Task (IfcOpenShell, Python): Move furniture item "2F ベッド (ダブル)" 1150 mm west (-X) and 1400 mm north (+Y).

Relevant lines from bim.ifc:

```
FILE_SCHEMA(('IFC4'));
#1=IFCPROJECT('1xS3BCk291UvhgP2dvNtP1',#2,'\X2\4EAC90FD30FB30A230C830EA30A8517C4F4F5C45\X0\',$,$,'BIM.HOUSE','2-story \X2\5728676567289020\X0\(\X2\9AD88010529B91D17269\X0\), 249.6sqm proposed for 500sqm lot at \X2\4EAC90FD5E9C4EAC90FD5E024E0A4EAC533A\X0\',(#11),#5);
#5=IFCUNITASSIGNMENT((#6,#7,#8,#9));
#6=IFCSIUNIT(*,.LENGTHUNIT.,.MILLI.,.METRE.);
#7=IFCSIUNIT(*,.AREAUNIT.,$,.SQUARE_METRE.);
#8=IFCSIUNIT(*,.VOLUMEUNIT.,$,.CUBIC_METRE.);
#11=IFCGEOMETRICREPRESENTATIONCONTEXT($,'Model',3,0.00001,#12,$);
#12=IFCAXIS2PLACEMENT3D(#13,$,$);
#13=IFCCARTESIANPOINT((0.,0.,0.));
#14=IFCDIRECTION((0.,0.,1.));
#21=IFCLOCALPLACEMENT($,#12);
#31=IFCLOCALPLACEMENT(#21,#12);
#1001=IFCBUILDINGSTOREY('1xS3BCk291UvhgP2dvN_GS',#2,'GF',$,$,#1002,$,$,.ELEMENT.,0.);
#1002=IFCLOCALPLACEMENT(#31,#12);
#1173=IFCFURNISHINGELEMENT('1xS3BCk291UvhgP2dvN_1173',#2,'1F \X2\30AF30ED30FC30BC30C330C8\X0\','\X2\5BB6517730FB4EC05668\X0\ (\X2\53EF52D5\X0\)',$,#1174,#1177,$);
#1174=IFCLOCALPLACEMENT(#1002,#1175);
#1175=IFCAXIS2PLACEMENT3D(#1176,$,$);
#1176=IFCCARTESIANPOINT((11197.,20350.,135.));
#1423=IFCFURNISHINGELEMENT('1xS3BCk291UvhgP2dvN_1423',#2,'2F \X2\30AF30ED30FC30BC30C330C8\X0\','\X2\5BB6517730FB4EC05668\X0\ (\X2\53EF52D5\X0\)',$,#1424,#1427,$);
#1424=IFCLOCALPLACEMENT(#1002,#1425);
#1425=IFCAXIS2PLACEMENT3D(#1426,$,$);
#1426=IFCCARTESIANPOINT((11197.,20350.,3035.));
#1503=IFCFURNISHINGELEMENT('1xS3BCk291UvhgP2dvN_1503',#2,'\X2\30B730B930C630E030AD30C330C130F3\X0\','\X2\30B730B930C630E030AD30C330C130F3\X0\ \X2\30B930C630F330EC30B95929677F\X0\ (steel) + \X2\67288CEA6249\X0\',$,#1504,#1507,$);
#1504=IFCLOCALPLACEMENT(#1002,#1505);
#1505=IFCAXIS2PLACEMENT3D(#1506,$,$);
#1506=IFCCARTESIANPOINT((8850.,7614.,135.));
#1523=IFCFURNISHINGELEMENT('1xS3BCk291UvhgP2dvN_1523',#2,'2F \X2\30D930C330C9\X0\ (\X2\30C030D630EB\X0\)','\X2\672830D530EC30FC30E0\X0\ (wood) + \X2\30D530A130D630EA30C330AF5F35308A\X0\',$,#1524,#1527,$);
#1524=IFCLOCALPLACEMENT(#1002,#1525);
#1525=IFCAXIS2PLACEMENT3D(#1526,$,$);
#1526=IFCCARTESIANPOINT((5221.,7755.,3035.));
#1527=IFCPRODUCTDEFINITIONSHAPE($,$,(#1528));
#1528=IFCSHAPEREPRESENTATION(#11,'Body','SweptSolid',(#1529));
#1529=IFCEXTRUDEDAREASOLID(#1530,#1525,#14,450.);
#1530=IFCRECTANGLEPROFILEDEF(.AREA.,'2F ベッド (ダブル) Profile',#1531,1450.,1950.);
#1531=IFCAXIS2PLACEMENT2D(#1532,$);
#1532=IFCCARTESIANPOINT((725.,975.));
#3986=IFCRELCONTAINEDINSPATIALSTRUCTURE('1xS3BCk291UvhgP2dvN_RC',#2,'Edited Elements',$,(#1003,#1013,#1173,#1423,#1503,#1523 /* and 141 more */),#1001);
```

```python
import ifcopenshell
import ifcopenshell.api.geometry
import ifcopenshell.util.placement
import ifcopenshell.util.unit

model = ifcopenshell.open("bim.ifc")
unit_scale = ifcopenshell.util.unit.calculate_unit_scale(model)

item = model.by_guid("1xS3BCk291UvhgP2dvN_1523")
matrix = ifcopenshell.util.placement.get_local_placement(item.ObjectPlacement)
matrix[0, 3] -= 1.15 / unit_scale
matrix[1, 3] += 1.4 / unit_scale
ifcopenshell.api.geometry.edit_object_placement(model, product=item, matrix=matrix, is_si=False)

print(ifcopenshell.util.placement.get_local_placement(item.ObjectPlacement).round(3) + 0.0)

model.write("bim_rev.ifc")
```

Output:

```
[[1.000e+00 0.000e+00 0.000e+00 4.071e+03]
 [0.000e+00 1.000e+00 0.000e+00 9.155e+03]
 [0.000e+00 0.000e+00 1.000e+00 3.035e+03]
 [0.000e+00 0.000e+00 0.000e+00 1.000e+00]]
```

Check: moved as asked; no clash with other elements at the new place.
